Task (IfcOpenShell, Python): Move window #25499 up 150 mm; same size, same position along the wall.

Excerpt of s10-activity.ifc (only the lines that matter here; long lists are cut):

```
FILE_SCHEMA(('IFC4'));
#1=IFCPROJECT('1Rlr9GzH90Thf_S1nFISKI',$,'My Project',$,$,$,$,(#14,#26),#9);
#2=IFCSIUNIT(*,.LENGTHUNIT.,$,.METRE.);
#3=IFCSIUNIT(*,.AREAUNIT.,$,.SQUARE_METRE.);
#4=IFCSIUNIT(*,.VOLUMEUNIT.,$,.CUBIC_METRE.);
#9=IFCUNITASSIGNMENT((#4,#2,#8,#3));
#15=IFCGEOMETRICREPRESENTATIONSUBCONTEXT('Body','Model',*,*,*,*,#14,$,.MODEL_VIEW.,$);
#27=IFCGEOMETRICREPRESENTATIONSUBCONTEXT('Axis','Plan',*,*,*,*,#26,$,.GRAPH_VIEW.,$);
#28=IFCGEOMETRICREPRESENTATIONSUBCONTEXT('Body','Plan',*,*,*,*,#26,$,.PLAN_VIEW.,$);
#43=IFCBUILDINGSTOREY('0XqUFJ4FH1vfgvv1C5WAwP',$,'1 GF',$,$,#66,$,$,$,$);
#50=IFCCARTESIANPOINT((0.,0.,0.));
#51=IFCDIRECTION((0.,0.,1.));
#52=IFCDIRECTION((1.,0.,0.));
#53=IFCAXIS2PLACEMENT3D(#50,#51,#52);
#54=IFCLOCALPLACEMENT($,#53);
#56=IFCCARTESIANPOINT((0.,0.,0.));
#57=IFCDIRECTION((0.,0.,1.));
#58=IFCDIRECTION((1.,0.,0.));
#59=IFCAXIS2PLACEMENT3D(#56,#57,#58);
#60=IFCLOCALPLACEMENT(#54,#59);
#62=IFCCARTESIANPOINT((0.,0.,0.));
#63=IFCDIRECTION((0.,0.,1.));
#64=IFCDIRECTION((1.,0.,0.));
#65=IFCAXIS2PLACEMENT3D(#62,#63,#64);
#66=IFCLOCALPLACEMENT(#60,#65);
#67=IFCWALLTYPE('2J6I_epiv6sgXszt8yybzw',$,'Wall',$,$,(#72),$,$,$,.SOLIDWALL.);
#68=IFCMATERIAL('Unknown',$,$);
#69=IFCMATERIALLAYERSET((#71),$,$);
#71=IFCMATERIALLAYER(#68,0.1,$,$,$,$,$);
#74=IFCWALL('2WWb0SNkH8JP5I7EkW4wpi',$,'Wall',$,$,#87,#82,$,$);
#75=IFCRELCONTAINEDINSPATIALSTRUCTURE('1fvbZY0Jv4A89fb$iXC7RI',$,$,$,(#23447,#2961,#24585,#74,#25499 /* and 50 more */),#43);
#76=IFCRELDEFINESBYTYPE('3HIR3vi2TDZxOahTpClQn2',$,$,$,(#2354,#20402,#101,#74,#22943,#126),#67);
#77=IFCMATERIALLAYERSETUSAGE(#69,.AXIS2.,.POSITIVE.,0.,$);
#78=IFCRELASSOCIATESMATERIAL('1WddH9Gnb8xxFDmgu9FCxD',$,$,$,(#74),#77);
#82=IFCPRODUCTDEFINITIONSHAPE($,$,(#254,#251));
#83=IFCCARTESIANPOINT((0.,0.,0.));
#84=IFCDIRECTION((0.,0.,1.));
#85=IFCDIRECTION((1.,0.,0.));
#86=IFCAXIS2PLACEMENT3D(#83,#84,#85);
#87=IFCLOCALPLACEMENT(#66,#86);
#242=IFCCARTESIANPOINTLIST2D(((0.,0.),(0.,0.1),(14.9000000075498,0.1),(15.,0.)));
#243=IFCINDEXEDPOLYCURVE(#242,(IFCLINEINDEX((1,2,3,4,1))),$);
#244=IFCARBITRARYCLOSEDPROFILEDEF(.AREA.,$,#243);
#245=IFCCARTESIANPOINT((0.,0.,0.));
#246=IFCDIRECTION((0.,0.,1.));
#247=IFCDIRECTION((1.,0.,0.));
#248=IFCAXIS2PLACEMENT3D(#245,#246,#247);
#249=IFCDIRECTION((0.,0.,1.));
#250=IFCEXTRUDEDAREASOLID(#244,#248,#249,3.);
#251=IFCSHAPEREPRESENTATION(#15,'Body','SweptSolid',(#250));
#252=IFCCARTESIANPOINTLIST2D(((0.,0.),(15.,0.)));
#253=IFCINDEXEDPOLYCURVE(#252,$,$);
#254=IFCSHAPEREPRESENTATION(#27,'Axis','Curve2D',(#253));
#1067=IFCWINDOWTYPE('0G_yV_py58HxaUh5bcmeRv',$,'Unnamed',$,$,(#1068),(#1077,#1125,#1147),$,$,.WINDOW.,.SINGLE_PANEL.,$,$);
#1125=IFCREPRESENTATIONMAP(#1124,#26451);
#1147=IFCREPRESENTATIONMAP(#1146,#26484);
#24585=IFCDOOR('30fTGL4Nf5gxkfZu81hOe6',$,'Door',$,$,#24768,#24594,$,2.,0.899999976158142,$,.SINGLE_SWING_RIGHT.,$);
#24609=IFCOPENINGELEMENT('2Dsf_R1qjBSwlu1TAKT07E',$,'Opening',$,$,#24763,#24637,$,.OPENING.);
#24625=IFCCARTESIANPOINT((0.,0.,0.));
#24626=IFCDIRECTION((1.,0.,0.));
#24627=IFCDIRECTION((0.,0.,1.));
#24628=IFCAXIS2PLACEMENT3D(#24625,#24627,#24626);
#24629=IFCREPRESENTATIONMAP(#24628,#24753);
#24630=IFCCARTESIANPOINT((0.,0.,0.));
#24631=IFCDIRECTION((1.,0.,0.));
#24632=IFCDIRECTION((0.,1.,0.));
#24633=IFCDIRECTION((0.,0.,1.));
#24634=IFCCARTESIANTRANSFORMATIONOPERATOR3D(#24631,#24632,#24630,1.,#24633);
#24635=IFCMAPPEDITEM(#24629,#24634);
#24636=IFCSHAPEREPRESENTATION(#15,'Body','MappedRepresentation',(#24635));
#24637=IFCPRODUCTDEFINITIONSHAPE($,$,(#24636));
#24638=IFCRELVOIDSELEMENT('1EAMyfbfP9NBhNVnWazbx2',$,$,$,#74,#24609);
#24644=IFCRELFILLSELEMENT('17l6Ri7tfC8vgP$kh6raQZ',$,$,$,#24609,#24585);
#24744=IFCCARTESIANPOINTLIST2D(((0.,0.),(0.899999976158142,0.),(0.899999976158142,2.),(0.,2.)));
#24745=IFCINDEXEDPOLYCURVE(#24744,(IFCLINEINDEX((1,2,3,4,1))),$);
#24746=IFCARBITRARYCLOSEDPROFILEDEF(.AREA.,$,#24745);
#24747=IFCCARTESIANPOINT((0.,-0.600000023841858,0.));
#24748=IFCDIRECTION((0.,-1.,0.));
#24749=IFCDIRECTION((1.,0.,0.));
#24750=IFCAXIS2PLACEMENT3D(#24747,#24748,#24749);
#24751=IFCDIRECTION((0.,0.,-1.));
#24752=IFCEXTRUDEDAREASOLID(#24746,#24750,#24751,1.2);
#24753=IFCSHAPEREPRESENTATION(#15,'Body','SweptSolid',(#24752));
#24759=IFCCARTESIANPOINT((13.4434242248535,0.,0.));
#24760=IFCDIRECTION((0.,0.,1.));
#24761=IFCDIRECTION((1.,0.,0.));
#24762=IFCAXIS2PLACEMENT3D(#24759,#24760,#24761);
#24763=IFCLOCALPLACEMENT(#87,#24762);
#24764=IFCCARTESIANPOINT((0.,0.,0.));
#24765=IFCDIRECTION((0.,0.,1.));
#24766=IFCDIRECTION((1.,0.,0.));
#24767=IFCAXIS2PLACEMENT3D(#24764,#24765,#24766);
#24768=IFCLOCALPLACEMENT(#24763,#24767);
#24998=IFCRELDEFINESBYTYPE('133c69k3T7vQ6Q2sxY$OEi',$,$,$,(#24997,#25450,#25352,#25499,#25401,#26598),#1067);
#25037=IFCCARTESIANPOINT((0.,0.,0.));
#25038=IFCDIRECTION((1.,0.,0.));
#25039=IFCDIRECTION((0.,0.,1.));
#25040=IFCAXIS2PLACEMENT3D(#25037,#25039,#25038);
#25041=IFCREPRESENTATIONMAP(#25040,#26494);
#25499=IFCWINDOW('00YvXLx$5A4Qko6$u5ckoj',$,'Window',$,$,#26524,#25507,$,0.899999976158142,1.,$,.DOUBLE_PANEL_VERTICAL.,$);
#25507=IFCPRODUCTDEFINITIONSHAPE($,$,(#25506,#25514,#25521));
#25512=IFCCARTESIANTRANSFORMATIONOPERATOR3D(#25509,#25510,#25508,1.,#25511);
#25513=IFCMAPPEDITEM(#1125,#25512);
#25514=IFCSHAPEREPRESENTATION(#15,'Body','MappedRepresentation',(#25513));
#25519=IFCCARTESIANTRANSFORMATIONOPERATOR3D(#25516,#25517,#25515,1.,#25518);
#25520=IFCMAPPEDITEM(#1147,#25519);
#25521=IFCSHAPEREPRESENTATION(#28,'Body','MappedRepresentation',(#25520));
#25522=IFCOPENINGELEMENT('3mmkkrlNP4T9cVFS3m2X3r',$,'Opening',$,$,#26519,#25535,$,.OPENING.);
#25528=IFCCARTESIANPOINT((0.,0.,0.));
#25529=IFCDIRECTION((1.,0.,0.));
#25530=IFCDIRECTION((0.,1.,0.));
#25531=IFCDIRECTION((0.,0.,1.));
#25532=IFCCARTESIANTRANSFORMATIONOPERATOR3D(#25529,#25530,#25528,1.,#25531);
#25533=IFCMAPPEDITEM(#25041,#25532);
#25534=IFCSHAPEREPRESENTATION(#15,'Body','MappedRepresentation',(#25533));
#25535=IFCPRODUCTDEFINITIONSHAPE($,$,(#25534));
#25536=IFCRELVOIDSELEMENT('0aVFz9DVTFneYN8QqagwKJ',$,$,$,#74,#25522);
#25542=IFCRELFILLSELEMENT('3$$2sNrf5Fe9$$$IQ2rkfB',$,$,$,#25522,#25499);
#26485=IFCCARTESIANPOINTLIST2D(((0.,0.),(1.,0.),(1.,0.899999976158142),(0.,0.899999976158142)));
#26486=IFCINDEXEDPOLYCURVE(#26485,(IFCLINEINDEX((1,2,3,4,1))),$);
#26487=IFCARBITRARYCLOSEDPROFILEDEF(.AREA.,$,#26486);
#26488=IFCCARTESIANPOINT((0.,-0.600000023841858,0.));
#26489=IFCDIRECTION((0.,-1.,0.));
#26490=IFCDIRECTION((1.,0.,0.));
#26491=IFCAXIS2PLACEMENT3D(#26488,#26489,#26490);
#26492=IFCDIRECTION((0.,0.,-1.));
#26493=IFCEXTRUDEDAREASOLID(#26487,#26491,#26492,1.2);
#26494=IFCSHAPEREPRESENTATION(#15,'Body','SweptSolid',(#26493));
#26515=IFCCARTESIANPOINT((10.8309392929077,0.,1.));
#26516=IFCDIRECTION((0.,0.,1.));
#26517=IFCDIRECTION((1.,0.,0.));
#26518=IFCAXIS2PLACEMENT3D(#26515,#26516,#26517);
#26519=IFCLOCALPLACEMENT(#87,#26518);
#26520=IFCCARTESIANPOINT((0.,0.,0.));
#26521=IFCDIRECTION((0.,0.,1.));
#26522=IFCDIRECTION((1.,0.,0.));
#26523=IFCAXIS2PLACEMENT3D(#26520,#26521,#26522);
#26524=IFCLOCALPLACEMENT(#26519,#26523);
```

```python
import numpy as np
import ifcopenshell
import ifcopenshell.api.geometry
import ifcopenshell.util.placement
import ifcopenshell.util.unit

model = ifcopenshell.open("s10-activity.ifc")
unit_scale = ifcopenshell.util.unit.calculate_unit_scale(model)

window = model.by_guid("00YvXLx$5A4Qko6$u5ckoj")
opening = window.FillsVoids[0].RelatingOpeningElement
dz = 0.15 / unit_scale

shift = np.array([0.0, 0.0, dz])
# The window is placed relative to its opening, so it follows when the opening moves.
matrix = ifcopenshell.util.placement.get_local_placement(opening.ObjectPlacement)
matrix[:3, 3] += shift
ifcopenshell.api.geometry.edit_object_placement(
    model, product=opening, matrix=matrix, is_si=False, should_transform_children=True
)

print(f"moved by {dz * unit_scale:+.3f} m")

model.write("s10-activity_v2.ifc")
```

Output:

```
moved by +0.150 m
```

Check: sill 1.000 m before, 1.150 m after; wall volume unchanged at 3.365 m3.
